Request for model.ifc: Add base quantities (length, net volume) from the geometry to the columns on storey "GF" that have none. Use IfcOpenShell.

First a look at what the model holds.

```python
import ifcopenshell
import ifcopenshell.util.element
import ifcopenshell.util.unit

model = ifcopenshell.open("model.ifc")
print(model.schema)
for unit_type in ("LENGTHUNIT", "AREAUNIT", "VOLUMEUNIT"):
    print(unit_type, ifcopenshell.util.unit.calculate_unit_scale(model, unit_type))
storey = next(s for s in model.by_type("IfcBuildingStorey") if s.Name == "GF")
columns = [e for e in ifcopenshell.util.element.get_decomposition(storey) if e.is_a("IfcColumn")]
for e in sorted(columns, key=lambda e: e.id()):
    print(e.id(), e.is_a(), e.Name, list(ifcopenshell.util.element.get_psets(e, qtos_only=True)), sep=" | ")
```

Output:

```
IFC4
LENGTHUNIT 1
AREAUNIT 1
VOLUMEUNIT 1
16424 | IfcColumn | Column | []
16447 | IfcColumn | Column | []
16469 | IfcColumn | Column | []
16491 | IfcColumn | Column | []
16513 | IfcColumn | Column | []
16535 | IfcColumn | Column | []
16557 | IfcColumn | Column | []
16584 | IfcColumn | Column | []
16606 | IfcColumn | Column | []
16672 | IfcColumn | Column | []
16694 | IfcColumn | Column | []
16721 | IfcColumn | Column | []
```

```python
import ifcopenshell
import ifcopenshell.api.pset
import ifcopenshell.geom
import ifcopenshell.util.element
import ifcopenshell.util.shape
import ifcopenshell.util.unit

model = ifcopenshell.open("model.ifc")
unit_scale = ifcopenshell.util.unit.calculate_unit_scale(model)
volume_scale = ifcopenshell.util.unit.calculate_unit_scale(model, "VOLUMEUNIT")
settings = ifcopenshell.geom.settings()

storey = next(s for s in model.by_type("IfcBuildingStorey") if s.Name == "GF")
columns = [e for e in ifcopenshell.util.element.get_decomposition(storey) if e.is_a("IfcColumn")]

for e in sorted(columns, key=lambda e: e.id()):
    if ifcopenshell.util.element.get_psets(e, qtos_only=True, should_inherit=False):
        continue
    # Geometry comes back in metres, in the element's own axes.
    shape = ifcopenshell.geom.create_shape(settings, e)
    values = {
        "Length": ifcopenshell.util.shape.get_z(shape.geometry) / unit_scale,
        "NetVolume": ifcopenshell.util.shape.get_volume(shape.geometry) / volume_scale,
    }
    qto = ifcopenshell.api.pset.add_qto(model, product=e, name="Qto_ColumnBaseQuantities")
    ifcopenshell.api.pset.edit_qto(model, qto=qto, properties=values)
    print(e.id(), {k: round(v, 3) for k, v in values.items()})

model.write("model_v2.ifc")
```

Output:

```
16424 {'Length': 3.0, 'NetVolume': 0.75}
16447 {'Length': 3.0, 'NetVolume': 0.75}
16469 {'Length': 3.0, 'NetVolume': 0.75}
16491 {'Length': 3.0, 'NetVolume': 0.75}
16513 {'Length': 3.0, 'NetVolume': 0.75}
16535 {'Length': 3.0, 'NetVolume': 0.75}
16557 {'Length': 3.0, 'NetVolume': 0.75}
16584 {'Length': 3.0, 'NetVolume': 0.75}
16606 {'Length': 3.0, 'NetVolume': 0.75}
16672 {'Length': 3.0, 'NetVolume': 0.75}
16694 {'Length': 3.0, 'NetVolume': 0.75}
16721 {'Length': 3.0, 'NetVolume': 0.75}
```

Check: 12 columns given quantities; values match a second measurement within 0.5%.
